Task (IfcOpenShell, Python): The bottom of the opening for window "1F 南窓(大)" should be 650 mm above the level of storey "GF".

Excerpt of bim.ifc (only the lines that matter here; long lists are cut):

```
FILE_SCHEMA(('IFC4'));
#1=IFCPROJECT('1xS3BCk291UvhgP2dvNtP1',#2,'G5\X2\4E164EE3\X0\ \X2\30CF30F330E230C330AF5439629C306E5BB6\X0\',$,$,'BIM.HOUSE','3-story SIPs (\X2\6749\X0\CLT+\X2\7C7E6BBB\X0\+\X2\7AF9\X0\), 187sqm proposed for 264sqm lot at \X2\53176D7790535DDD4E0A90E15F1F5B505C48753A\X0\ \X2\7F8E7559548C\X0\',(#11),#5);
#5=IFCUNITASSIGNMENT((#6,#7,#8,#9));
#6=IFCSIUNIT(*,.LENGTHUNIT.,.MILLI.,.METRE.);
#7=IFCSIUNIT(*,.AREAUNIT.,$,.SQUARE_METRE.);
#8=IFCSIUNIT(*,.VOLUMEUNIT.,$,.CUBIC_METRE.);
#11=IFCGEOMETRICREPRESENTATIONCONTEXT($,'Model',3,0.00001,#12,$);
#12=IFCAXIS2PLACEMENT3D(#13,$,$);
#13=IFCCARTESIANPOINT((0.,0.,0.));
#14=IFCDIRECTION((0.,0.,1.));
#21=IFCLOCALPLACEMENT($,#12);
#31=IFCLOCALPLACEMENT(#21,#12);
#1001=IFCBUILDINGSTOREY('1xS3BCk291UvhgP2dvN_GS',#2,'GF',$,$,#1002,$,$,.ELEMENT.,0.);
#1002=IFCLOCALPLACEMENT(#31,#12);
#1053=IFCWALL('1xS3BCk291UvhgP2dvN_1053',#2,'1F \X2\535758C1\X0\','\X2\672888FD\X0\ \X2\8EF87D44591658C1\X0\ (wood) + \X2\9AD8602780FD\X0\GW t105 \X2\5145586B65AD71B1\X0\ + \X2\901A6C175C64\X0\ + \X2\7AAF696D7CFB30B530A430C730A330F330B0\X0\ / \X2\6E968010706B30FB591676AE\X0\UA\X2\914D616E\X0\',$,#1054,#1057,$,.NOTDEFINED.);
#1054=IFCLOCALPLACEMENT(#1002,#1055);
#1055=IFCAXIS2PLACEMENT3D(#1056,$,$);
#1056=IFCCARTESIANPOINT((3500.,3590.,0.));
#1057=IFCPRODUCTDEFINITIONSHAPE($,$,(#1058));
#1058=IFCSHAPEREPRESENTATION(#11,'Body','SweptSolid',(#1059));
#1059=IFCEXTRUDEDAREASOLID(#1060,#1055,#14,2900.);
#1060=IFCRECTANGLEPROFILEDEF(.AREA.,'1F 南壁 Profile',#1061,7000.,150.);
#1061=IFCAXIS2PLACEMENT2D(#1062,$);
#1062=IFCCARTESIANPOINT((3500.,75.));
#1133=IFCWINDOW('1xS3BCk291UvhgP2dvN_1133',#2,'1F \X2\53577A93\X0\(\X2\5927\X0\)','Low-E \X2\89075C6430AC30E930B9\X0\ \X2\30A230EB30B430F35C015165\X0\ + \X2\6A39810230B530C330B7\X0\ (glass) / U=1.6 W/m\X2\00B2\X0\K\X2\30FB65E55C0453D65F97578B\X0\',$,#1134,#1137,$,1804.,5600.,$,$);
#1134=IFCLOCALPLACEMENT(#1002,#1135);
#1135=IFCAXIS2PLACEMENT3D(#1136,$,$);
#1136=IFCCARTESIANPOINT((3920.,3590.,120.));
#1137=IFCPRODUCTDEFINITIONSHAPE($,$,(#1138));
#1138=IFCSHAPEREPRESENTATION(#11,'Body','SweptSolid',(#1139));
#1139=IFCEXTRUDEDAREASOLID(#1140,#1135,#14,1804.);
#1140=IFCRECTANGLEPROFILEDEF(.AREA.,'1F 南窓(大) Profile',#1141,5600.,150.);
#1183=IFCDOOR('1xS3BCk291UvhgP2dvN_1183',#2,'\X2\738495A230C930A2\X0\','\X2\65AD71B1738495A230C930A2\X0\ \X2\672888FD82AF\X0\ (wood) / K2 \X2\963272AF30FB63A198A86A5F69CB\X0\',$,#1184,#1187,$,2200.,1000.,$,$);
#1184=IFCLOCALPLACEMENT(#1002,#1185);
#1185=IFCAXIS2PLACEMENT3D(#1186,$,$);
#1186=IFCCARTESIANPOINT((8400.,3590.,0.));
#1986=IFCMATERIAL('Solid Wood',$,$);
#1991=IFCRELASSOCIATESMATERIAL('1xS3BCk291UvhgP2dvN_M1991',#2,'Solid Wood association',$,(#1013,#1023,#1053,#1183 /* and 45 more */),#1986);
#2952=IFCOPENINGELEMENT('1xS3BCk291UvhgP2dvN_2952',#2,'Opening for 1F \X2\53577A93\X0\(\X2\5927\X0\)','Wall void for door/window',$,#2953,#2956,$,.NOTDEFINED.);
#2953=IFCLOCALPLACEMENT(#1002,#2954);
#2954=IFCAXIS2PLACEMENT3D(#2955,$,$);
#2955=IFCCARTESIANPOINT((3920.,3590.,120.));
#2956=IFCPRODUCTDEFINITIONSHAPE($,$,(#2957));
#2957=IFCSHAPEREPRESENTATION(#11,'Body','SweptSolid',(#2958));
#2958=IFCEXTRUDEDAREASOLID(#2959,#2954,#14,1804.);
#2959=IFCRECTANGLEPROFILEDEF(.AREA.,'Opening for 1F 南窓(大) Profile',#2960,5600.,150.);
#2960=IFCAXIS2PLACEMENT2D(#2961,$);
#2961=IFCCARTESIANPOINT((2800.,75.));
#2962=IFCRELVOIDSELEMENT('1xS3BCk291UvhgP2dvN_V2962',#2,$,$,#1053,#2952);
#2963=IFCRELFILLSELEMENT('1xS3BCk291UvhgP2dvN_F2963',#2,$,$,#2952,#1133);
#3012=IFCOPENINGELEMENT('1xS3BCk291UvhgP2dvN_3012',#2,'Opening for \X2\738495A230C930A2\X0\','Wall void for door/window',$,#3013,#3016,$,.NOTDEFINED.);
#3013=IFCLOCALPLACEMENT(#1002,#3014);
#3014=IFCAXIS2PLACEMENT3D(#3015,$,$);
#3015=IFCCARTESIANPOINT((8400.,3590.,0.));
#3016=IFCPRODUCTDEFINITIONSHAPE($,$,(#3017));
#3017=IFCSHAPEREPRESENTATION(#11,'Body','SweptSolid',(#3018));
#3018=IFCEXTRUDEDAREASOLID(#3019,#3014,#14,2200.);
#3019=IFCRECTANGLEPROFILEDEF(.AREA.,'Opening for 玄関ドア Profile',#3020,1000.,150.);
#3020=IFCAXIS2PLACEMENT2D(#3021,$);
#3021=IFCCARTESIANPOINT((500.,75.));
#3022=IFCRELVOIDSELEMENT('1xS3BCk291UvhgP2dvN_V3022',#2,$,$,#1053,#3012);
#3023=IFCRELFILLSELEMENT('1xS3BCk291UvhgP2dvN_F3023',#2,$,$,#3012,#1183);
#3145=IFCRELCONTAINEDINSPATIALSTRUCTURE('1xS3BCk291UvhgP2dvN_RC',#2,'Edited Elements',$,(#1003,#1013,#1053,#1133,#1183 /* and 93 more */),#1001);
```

```python
import numpy as np
import ifcopenshell
import ifcopenshell.api.geometry
import ifcopenshell.geom
import ifcopenshell.util.element
import ifcopenshell.util.placement
import ifcopenshell.util.shape
import ifcopenshell.util.unit

model = ifcopenshell.open("bim.ifc")
unit_scale = ifcopenshell.util.unit.calculate_unit_scale(model)

window = model.by_id(1133)
opening = window.FillsVoids[0].RelatingOpeningElement
storey = ifcopenshell.util.element.get_container(window, ifc_class="IfcBuildingStorey")
level = ifcopenshell.util.placement.get_local_placement(storey.ObjectPlacement)[2, 3]

# The opening's origin need not be at the sill, so measure its lowest point.
shape = ifcopenshell.geom.create_shape(ifcopenshell.geom.settings(), opening)
bottom = ifcopenshell.util.shape.get_shape_bottom_elevation(shape, shape.geometry) / unit_scale
dz = level + 0.65 / unit_scale - bottom

shift = np.array([0.0, 0.0, dz])
# The window is not placed relative to its opening, so move both.
for product in (opening, window):
    matrix = ifcopenshell.util.placement.get_local_placement(product.ObjectPlacement)
    matrix[:3, 3] += shift
    ifcopenshell.api.geometry.edit_object_placement(model, product=product, matrix=matrix, is_si=False)

print(f"moved by {dz * unit_scale:+.3f} m")

model.write("bim_edited.ifc")
```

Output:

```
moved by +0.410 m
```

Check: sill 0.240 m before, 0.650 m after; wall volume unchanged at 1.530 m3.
